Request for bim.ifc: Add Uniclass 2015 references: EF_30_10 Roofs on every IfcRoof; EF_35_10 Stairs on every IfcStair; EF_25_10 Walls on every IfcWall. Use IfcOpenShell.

First a look at what the model holds.

```python
import ifcopenshell

model = ifcopenshell.open("bim.ifc")
print(model.schema)
print("classifications:", [c.Name for c in model.by_type("IfcClassification")])
for ifc_class in ("IfcDoor", "IfcRoof", "IfcStair", "IfcWall", "IfcWindow"):
    print(ifc_class, len(model.by_type(ifc_class)))
```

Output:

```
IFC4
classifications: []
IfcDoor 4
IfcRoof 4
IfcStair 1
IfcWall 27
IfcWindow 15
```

```python
import ifcopenshell
import ifcopenshell.api.classification

model = ifcopenshell.open("bim.ifc")

system = ifcopenshell.api.classification.add_classification(model, classification="Uniclass 2015")

codes = {
    "IfcRoof": ("EF_30_10", "Roofs"),
    "IfcStair": ("EF_35_10", "Stairs"),
    "IfcWall": ("EF_25_10", "Walls"),
}
for ifc_class, (code, name) in codes.items():
    products = model.by_type(ifc_class)
    ifcopenshell.api.classification.add_reference(
        model, products=products, classification=system, identification=code, name=name
    )
    print(code, len(products))

model.write("bim_rev.ifc")
```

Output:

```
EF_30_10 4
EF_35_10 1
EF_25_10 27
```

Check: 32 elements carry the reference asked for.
